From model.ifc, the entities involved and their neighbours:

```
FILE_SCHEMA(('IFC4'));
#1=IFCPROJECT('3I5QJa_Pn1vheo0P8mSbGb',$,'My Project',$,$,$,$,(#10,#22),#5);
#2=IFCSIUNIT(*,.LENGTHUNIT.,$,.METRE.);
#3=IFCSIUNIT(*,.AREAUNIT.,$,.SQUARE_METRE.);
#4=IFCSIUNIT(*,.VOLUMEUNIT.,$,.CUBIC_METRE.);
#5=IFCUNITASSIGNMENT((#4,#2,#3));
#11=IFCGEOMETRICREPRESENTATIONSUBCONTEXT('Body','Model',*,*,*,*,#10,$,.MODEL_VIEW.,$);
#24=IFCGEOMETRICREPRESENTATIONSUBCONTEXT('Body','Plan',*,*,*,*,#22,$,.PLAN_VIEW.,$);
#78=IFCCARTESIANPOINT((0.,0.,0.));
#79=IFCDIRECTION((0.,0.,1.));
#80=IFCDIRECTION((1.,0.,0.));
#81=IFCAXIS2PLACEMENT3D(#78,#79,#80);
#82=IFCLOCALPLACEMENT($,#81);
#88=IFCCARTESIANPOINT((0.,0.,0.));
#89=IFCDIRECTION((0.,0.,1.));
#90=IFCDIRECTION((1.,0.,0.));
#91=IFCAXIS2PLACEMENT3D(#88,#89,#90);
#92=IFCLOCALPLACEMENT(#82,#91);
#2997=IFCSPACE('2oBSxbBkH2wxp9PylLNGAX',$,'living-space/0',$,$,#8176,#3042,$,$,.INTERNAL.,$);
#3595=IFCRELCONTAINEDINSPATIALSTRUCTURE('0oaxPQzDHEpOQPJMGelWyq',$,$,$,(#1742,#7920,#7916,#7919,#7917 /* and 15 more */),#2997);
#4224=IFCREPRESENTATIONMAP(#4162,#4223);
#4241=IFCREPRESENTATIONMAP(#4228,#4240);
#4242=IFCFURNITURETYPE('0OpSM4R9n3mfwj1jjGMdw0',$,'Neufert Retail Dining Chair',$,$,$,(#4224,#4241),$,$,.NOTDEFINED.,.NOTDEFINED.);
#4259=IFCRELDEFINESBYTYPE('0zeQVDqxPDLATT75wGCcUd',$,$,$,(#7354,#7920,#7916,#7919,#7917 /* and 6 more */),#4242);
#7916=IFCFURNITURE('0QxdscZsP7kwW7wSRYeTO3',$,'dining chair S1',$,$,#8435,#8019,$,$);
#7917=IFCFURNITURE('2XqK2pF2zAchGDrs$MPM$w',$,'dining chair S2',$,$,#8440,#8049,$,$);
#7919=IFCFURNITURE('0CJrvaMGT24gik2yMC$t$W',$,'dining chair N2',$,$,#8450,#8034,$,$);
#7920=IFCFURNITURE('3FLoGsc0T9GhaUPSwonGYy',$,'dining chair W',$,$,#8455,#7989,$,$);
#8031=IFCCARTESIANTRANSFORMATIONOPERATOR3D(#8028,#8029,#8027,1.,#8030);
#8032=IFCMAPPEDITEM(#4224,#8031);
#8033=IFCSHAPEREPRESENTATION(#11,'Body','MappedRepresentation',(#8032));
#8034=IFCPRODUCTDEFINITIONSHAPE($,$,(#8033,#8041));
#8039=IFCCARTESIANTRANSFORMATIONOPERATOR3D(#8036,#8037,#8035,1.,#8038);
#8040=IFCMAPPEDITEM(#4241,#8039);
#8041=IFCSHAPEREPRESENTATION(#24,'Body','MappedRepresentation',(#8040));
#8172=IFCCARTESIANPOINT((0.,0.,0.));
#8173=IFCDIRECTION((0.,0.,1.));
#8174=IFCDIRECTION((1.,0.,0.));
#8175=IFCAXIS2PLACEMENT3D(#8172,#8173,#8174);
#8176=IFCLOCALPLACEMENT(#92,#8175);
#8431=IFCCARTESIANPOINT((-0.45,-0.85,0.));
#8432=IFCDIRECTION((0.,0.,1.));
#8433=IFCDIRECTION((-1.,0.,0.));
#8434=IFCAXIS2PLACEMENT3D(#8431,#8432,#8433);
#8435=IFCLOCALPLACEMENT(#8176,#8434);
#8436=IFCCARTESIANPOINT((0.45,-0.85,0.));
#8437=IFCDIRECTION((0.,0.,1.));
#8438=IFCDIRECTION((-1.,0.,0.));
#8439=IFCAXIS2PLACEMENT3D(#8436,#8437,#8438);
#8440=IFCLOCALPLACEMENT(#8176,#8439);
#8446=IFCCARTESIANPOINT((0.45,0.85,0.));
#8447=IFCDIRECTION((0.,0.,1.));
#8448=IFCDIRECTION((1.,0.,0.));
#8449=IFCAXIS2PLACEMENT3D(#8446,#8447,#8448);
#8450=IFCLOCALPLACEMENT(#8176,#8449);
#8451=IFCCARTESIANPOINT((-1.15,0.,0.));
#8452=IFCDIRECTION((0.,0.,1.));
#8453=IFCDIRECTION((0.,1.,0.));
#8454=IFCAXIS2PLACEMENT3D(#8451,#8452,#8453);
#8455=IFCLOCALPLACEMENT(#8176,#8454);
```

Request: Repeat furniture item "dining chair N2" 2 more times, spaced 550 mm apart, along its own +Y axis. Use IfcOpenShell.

```python
import ifcopenshell
import ifcopenshell.api.geometry
import ifcopenshell.api.root
import ifcopenshell.util.element
import ifcopenshell.util.placement
import ifcopenshell.util.unit

model = ifcopenshell.open("model.ifc")
unit_scale = ifcopenshell.util.unit.calculate_unit_scale(model)

source = model.by_guid("0CJrvaMGT24gik2yMC$t$W")
base = ifcopenshell.util.placement.get_local_placement(source.ObjectPlacement)
step = base[:3, 1] * 0.55 / unit_scale

for i in range(1, 3):
    copy = ifcopenshell.api.root.copy_class(model, product=source)
    copy.Representation = ifcopenshell.util.element.copy_deep(
        model, source.Representation, exclude=["IfcGeometricRepresentationContext", "IfcRepresentationMap"]
    )
    matrix = base.copy()
    matrix[:3, 3] += i * step
    print("added at", matrix[:3, 3].round(3) + 0.0)
    ifcopenshell.api.geometry.edit_object_placement(model, product=copy, matrix=matrix, is_si=False)

model.write("model-out.ifc")
```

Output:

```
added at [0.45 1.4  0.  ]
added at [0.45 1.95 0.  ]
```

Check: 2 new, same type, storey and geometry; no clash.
